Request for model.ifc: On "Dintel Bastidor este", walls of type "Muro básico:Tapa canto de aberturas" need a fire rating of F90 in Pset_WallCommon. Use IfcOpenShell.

First a look at what the model holds.

```python
import ifcopenshell
import ifcopenshell.util.element

model = ifcopenshell.open("model.ifc")
print(model.schema)
storey = next(s for s in model.by_type("IfcBuildingStorey") if s.Name == "Dintel Bastidor este")
walls = [e for e in ifcopenshell.util.element.get_decomposition(storey) if e.is_a("IfcWall")]
seen = {}
for e in walls:
    element_type = ifcopenshell.util.element.get_type(e)
    key = (element_type.Name if element_type != e and element_type else None, ifcopenshell.util.element.get_pset(e, "Pset_WallCommon", "FireRating"))
    seen[key] = seen.get(key, 0) + 1
for (name, value), count in sorted(seen.items(), key=str):
    print(count, "x", name, "|", value)
```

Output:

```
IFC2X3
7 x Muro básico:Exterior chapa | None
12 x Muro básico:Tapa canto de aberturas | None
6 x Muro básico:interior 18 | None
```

```python
import ifcopenshell
import ifcopenshell.api.pset
import ifcopenshell.util.element

model = ifcopenshell.open("model.ifc")

storey = next(s for s in model.by_type("IfcBuildingStorey") if s.Name == "Dintel Bastidor este")
walls = [e for e in ifcopenshell.util.element.get_decomposition(storey) if e.is_a("IfcWall")]

count = 0
for e in walls:
    element_type = ifcopenshell.util.element.get_type(e)
    if element_type in (None, e) or element_type.Name != "Muro básico:Tapa canto de aberturas":
        continue
    # add_pset returns the element's existing set when there is one.
    pset = ifcopenshell.api.pset.add_pset(model, product=e, name="Pset_WallCommon")
    ifcopenshell.api.pset.edit_pset(model, pset=pset, properties={"FireRating": "F90"})
    count += 1

print(count, "walls updated")

model.write("model_rev.ifc")
```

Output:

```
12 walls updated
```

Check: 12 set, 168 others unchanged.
